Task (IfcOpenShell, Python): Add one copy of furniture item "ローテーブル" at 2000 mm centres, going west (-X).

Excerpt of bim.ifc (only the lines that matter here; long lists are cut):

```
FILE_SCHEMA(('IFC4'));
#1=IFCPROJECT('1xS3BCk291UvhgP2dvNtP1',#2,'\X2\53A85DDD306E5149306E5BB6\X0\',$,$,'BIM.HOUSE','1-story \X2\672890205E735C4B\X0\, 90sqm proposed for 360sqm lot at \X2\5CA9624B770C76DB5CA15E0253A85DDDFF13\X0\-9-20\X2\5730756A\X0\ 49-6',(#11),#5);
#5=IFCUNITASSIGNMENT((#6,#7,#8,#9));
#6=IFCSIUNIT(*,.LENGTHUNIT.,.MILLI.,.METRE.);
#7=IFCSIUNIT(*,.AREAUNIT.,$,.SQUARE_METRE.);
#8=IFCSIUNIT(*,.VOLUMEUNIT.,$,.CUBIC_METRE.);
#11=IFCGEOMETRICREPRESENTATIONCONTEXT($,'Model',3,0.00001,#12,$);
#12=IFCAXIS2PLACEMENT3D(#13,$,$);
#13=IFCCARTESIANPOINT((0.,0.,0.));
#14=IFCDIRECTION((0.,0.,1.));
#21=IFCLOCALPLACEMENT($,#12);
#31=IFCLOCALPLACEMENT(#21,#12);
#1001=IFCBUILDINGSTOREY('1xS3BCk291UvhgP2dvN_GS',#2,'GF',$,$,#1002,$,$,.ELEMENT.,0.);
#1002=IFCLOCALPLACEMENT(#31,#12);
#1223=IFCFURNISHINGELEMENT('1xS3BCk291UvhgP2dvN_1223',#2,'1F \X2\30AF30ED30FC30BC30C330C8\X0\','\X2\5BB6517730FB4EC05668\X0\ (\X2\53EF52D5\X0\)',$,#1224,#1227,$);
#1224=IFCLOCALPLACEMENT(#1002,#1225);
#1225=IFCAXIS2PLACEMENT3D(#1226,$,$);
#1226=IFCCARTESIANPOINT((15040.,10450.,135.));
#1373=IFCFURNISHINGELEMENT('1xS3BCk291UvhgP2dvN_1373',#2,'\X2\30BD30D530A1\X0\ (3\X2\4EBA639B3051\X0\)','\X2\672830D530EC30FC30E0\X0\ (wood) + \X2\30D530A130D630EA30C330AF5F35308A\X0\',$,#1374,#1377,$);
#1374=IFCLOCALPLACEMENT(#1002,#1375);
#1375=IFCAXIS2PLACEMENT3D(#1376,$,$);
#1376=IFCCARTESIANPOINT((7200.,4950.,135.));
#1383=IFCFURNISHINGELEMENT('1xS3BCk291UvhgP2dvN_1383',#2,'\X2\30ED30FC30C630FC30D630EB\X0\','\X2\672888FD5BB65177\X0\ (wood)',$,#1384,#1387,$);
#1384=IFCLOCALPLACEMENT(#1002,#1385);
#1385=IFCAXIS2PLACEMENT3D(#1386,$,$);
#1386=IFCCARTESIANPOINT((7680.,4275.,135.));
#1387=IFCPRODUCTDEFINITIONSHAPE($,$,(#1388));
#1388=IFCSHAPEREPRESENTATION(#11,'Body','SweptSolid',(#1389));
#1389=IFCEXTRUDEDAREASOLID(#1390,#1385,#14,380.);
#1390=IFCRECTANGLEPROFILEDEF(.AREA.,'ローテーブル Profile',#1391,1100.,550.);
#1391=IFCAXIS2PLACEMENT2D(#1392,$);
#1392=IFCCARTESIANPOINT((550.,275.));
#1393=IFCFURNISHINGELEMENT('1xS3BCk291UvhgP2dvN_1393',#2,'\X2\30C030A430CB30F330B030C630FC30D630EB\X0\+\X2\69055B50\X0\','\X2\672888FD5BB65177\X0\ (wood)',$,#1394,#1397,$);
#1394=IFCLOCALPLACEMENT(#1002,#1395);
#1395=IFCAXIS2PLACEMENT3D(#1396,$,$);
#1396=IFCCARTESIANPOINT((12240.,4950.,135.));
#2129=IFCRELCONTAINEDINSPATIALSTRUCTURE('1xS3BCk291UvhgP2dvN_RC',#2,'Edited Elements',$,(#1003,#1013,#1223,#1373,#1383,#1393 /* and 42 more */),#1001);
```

```python
import numpy as np
import ifcopenshell
import ifcopenshell.api.geometry
import ifcopenshell.api.root
import ifcopenshell.util.element
import ifcopenshell.util.placement

model = ifcopenshell.open("bim.ifc")


def reuse_history(source, copy):
    """copy_class also copies each property set's owner history, people and application; keep the originals."""
    for rel in copy.IsDefinedBy:
        if rel.is_a("IfcRelDefinesByProperties") and (history := rel.RelatingPropertyDefinition.OwnerHistory):
            rel.RelatingPropertyDefinition.OwnerHistory = source.OwnerHistory
            ifcopenshell.util.element.remove_deep2(model, history)


source = model.by_guid("1xS3BCk291UvhgP2dvN_1383")
base = ifcopenshell.util.placement.get_local_placement(source.ObjectPlacement)
step = np.array([-1.0, 0.0, 0.0]) * 2000.0

for i in range(1, 2):
    copy = ifcopenshell.api.root.copy_class(model, product=source)
    copy.Representation = ifcopenshell.util.element.copy_deep(
        model, source.Representation, exclude=["IfcGeometricRepresentationContext", "IfcRepresentationMap"]
    )
    reuse_history(source, copy)
    matrix = base.copy()
    matrix[:3, 3] += i * step
    print("added at", matrix[:3, 3].round(3) + 0.0)
    ifcopenshell.api.geometry.edit_object_placement(model, product=copy, matrix=matrix, is_si=False)

model.write("bim_rev.ifc")
```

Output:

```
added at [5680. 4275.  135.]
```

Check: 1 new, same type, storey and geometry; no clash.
